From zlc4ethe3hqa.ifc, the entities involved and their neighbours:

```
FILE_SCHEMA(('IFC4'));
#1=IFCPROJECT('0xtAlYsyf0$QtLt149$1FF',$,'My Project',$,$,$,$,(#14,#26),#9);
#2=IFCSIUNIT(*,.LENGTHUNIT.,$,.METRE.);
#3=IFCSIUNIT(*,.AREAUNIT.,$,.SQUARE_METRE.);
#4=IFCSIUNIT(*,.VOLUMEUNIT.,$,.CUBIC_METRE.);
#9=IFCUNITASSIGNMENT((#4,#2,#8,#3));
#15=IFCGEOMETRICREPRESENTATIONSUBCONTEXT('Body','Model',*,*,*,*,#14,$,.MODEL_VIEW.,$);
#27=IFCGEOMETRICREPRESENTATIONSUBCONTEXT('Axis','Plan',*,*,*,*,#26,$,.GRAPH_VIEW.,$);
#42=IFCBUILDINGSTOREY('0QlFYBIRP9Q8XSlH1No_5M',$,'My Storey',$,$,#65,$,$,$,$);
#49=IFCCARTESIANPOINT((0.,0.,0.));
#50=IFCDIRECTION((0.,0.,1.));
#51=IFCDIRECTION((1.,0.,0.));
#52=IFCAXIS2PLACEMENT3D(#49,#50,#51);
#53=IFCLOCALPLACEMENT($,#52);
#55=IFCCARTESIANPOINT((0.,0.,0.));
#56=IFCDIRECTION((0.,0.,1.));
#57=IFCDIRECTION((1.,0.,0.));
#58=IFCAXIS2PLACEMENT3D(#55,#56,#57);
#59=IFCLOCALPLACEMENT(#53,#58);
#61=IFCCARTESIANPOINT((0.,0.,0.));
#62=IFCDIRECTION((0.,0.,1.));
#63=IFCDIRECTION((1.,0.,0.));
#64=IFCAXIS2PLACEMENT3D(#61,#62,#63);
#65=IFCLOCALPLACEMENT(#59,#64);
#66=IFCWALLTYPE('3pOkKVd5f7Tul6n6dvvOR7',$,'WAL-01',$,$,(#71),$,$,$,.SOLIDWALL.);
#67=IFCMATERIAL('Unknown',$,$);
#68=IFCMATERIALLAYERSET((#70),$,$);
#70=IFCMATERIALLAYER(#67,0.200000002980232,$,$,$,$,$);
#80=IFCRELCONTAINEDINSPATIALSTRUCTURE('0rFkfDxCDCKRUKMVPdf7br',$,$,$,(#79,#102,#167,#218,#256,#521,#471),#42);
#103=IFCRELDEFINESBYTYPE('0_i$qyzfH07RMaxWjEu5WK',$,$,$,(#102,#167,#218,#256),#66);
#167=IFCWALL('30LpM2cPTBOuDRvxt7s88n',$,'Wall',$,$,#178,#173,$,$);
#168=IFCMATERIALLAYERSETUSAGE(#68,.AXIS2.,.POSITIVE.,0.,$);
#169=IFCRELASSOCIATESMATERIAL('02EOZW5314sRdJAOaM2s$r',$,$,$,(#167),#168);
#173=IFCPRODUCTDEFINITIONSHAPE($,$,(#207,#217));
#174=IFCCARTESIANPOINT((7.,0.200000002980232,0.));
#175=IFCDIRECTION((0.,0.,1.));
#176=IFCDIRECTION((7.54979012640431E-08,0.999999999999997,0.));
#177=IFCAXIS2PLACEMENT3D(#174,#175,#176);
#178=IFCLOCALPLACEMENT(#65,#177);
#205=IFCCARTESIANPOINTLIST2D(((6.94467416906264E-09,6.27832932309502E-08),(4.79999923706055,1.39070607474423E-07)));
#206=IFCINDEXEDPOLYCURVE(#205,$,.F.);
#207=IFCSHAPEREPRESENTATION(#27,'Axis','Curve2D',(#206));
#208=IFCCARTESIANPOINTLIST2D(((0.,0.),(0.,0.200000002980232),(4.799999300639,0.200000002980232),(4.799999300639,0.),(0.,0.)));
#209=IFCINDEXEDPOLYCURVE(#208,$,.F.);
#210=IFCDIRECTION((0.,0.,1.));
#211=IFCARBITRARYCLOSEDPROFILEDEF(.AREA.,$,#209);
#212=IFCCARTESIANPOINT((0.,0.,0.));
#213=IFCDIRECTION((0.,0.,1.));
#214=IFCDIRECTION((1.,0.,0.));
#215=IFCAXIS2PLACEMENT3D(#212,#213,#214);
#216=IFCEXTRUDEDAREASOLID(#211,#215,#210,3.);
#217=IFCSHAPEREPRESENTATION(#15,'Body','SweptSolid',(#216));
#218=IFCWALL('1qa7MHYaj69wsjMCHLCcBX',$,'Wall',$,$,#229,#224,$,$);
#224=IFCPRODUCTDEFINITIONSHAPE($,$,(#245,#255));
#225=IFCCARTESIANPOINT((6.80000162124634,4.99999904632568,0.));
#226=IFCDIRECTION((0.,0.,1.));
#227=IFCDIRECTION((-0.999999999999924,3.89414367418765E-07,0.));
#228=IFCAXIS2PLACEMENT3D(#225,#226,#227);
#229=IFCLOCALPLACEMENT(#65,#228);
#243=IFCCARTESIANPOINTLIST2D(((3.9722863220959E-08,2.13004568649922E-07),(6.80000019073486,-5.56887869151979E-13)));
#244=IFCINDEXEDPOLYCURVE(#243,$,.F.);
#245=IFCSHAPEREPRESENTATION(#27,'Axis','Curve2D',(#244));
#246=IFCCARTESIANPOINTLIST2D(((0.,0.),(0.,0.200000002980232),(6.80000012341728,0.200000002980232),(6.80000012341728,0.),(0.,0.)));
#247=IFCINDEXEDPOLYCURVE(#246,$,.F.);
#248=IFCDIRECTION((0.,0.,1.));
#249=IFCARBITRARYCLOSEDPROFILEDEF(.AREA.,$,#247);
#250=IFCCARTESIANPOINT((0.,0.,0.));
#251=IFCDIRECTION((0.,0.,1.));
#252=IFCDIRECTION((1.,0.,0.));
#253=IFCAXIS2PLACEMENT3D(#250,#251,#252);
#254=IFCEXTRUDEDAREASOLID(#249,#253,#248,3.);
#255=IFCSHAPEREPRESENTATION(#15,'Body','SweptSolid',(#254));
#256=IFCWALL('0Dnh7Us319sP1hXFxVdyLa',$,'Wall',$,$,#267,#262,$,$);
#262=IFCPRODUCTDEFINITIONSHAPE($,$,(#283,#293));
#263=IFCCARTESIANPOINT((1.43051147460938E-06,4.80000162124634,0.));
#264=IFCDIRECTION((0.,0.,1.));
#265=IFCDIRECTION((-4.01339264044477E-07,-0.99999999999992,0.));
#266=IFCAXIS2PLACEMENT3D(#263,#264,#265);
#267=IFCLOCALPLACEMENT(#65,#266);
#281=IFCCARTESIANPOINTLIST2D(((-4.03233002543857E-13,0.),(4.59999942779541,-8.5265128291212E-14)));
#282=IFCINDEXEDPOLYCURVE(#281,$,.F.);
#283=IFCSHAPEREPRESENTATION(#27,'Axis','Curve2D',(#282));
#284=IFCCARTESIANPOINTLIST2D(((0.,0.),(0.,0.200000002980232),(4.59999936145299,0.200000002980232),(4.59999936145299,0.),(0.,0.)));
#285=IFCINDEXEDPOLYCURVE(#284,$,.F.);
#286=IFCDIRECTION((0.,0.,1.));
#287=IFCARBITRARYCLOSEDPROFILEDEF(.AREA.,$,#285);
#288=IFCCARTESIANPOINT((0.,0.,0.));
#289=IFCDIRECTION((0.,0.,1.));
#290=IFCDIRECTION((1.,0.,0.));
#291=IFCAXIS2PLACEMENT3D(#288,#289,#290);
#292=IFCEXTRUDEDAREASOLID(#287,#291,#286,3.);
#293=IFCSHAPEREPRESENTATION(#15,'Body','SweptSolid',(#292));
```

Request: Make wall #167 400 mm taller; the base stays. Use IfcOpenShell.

```python
import ifcopenshell
import ifcopenshell.geom
import ifcopenshell.util.representation
import ifcopenshell.util.shape

model = ifcopenshell.open("zlc4ethe3hqa.ifc")
settings = ifcopenshell.geom.settings()


def volume(element):
    """Net volume in cubic metres, openings subtracted."""
    shape = ifcopenshell.geom.create_shape(settings, element)
    return ifcopenshell.util.shape.get_volume(shape.geometry)


wall = model.by_guid("30LpM2cPTBOuDRvxt7s88n")
before = volume(wall)

body = ifcopenshell.util.representation.get_representation(wall, "Model", "Body")
solid = body.Items[0]
old_height = solid.Depth
solid.Depth += 0.4
after = volume(wall)

print(f"height {old_height:g} -> {solid.Depth:g}, volume {before:.3f} -> {after:.3f} m3")

model.write("zlc4ethe3hqa_v2.ifc")
```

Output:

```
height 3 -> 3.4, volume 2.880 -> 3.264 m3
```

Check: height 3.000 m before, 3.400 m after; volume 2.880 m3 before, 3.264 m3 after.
